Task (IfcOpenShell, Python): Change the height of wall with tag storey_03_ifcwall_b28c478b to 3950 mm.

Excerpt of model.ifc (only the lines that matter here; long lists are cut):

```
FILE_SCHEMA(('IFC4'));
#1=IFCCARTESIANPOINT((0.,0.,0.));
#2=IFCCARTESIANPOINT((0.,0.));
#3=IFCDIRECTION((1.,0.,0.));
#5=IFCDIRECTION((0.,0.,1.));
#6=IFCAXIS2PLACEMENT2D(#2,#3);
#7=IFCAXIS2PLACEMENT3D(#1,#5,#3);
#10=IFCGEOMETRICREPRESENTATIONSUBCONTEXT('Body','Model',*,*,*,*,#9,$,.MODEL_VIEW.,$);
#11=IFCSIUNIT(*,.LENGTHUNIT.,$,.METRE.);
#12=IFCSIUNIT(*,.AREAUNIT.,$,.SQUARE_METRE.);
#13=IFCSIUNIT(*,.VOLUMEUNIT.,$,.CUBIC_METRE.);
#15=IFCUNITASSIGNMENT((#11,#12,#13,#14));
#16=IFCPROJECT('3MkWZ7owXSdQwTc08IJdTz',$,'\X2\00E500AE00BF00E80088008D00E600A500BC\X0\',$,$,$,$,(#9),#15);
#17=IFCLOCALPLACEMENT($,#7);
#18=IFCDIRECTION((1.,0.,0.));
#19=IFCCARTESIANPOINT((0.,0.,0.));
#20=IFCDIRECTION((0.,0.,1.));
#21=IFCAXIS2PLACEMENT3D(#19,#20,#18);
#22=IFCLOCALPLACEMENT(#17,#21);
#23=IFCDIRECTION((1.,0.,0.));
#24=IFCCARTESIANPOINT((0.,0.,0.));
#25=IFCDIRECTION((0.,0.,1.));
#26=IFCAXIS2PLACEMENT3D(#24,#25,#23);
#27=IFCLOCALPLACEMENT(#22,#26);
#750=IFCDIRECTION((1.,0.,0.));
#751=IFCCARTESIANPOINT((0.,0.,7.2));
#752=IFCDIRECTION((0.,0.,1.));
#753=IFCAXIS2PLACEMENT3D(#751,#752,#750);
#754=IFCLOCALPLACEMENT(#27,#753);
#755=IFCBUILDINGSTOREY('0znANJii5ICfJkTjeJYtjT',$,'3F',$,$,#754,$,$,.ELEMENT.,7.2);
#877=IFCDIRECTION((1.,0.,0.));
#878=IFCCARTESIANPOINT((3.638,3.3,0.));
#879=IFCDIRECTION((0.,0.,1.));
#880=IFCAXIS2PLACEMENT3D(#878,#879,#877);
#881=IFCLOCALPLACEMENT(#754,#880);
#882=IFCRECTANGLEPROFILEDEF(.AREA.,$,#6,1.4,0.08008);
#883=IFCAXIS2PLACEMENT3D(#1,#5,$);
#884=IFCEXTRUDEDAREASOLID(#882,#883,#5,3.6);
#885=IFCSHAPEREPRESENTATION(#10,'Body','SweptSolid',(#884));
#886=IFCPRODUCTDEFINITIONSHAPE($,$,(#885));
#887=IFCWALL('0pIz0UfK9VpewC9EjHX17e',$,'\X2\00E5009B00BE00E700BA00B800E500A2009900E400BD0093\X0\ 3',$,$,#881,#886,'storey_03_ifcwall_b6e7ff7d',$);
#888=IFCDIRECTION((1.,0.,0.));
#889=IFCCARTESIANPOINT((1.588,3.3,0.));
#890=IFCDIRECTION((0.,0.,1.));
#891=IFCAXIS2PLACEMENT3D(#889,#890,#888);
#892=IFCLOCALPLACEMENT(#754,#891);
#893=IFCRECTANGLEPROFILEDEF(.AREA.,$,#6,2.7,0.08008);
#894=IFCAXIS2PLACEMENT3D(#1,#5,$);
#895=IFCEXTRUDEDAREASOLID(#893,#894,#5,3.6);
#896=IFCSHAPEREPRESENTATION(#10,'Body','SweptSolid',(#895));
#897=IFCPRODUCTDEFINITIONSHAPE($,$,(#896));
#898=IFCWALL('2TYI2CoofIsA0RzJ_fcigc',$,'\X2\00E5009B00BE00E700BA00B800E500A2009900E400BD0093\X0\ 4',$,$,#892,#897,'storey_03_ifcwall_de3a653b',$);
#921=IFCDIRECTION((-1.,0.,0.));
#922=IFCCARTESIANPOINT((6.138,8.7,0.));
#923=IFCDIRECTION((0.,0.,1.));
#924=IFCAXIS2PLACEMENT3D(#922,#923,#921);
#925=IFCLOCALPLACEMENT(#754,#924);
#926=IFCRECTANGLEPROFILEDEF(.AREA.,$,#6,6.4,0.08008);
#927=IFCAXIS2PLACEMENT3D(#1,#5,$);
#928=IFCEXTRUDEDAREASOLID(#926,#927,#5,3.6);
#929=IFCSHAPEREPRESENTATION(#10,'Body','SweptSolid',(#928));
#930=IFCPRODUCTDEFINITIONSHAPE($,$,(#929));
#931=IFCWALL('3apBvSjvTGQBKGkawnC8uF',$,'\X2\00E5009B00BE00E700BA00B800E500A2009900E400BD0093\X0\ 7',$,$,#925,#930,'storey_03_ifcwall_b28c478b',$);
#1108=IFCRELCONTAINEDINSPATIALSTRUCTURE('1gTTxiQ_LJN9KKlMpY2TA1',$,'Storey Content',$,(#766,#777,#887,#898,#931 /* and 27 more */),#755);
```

```python
import ifcopenshell
import ifcopenshell.geom
import ifcopenshell.util.representation
import ifcopenshell.util.shape
import ifcopenshell.util.unit

model = ifcopenshell.open("model.ifc")
unit_scale = ifcopenshell.util.unit.calculate_unit_scale(model)
settings = ifcopenshell.geom.settings()


def volume(element):
    """Net volume in cubic metres, openings subtracted."""
    shape = ifcopenshell.geom.create_shape(settings, element)
    return ifcopenshell.util.shape.get_volume(shape.geometry)


wall = model.by_guid("3apBvSjvTGQBKGkawnC8uF")
before = volume(wall)

body = ifcopenshell.util.representation.get_representation(wall, "Model", "Body")
solid = body.Items[0]
old_height = solid.Depth
solid.Depth = 3.95 / unit_scale
after = volume(wall)

print(f"height {old_height:g} -> {solid.Depth:g}, volume {before:.3f} -> {after:.3f} m3")

model.write("model_v2.ifc")
```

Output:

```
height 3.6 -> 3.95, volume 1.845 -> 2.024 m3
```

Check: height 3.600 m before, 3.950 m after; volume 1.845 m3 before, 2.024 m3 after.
